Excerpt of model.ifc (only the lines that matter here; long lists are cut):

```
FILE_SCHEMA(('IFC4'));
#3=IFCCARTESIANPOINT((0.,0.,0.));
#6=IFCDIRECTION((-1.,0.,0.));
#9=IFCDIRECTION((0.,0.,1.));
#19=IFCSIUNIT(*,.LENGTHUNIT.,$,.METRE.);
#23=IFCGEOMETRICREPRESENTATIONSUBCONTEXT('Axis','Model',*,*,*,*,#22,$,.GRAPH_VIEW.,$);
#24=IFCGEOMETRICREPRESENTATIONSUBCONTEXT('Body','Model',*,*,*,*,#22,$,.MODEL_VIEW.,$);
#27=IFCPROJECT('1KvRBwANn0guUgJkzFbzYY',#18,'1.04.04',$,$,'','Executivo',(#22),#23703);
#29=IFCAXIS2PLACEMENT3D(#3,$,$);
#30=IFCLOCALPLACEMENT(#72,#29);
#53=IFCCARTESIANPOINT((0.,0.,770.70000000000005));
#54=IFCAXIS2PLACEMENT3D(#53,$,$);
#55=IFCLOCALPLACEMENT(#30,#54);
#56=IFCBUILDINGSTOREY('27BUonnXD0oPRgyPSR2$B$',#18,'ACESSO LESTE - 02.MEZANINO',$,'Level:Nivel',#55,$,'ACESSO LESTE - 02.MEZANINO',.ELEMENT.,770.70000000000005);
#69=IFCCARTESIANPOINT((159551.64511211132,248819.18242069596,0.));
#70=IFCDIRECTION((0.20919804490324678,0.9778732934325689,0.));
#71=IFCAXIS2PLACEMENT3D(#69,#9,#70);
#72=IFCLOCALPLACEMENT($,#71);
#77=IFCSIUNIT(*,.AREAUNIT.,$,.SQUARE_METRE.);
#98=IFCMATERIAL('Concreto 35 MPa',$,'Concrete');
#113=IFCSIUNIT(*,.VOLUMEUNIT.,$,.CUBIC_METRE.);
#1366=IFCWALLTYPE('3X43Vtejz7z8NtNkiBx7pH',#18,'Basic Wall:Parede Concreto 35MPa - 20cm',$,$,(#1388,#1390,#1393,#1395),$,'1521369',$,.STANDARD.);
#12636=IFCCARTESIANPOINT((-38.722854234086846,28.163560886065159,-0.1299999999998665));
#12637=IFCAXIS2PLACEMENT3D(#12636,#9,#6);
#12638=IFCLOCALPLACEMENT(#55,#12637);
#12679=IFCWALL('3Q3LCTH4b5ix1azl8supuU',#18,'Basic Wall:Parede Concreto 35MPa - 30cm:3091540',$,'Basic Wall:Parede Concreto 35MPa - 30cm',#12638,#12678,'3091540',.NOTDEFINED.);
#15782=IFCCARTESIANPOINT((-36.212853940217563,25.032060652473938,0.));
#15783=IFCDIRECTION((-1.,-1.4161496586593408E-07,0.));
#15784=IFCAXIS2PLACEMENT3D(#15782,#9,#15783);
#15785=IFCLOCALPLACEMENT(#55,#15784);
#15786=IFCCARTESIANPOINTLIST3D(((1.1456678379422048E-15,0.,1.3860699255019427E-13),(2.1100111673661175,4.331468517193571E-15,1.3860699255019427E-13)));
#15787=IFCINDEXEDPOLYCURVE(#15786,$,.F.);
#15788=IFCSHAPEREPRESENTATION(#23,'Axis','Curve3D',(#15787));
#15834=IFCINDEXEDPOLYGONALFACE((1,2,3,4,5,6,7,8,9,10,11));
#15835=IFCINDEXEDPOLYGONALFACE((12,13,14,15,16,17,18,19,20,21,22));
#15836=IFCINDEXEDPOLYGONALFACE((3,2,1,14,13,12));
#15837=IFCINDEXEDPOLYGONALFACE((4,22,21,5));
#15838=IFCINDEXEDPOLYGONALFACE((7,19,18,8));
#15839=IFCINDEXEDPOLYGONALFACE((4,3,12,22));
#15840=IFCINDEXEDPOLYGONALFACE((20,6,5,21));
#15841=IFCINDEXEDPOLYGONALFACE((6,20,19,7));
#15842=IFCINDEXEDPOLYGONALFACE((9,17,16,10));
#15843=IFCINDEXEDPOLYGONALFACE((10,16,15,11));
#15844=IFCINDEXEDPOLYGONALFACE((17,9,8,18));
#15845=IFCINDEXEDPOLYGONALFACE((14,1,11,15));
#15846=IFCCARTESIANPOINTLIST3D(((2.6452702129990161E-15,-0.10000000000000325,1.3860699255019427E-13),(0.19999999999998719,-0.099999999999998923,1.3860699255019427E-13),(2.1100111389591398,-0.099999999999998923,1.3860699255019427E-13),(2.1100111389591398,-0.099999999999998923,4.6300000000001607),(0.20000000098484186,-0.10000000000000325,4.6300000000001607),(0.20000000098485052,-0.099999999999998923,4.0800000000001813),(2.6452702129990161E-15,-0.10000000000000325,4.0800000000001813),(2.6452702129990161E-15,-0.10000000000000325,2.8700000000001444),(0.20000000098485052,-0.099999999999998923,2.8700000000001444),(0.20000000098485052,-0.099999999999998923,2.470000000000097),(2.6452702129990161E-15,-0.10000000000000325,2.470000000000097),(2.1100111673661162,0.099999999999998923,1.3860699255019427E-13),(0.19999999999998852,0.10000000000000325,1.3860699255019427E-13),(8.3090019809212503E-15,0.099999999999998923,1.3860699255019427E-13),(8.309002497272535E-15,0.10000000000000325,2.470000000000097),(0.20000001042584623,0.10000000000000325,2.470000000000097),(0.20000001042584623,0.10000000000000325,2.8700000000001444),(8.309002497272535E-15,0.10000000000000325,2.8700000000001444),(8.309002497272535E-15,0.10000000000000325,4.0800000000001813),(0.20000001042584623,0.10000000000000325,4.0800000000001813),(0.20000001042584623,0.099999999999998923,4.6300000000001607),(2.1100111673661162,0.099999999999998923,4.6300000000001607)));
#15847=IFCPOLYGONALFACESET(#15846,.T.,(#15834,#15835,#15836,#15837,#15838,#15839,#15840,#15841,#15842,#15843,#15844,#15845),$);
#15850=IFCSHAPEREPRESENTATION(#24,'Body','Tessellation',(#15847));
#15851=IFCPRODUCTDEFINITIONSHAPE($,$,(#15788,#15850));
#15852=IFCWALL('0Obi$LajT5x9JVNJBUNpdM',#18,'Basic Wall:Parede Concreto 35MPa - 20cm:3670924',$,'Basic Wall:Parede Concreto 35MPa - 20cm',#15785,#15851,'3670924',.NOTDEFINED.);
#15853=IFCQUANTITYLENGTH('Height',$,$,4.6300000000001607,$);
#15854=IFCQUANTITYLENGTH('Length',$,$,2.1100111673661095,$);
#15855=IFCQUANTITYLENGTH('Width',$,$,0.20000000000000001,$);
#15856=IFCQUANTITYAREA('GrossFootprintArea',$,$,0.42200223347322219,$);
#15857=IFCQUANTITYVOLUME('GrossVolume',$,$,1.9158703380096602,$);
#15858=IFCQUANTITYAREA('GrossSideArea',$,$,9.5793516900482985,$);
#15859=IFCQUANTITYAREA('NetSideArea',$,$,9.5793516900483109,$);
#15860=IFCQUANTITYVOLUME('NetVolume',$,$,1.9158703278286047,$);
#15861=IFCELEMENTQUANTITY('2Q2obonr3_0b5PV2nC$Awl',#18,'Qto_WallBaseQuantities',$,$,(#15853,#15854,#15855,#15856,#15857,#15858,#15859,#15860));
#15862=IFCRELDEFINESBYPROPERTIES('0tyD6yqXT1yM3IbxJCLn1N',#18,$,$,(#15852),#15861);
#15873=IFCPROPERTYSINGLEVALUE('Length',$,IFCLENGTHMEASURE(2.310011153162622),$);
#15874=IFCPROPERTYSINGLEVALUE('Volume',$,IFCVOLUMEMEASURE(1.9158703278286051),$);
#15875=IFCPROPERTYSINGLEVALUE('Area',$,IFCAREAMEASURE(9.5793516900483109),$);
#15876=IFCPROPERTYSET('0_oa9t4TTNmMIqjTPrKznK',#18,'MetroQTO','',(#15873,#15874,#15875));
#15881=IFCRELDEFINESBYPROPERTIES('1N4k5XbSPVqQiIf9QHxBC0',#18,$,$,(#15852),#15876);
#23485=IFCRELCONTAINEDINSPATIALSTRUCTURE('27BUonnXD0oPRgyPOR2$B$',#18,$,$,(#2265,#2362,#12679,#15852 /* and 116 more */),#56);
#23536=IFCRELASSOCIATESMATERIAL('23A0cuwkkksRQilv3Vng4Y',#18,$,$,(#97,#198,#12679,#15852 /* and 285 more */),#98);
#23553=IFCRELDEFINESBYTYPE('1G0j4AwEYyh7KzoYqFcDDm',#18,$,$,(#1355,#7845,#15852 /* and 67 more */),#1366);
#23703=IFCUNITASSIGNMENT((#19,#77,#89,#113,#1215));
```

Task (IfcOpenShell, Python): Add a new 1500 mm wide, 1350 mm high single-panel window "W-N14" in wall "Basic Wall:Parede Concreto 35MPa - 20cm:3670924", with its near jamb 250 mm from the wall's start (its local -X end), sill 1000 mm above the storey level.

```python
import numpy as np
import ifcopenshell
import ifcopenshell.api.feature
import ifcopenshell.api.geometry
import ifcopenshell.api.pset
import ifcopenshell.api.root
import ifcopenshell.api.spatial
import ifcopenshell.geom
import ifcopenshell.util.element
import ifcopenshell.util.placement
import ifcopenshell.util.representation
import ifcopenshell.util.shape
import ifcopenshell.util.unit

model = ifcopenshell.open("model.ifc")
unit_scale = ifcopenshell.util.unit.calculate_unit_scale(model)
area_scale = ifcopenshell.util.unit.calculate_unit_scale(model, "AREAUNIT")
volume_scale = ifcopenshell.util.unit.calculate_unit_scale(model, "VOLUMEUNIT")
settings = ifcopenshell.geom.settings()


def volume(element):
    """Net volume in cubic metres, openings subtracted."""
    shape = ifcopenshell.geom.create_shape(settings, element)
    return ifcopenshell.util.shape.get_volume(shape.geometry)


wall = model.by_id(15852)
storey = ifcopenshell.util.element.get_container(wall, ifc_class="IfcBuildingStorey")
context = ifcopenshell.util.representation.get_context(model, "Model", "Body", "MODEL_VIEW")
before = volume(wall)

width, height, from_end, sill = 1.5, 1.35, 0.25, 1  # metres

# The wall runs along its own X axis, and the end named is its -X end.
wall_shape = ifcopenshell.geom.create_shape(settings, wall)
x, y, z = ifcopenshell.util.shape.get_vertices(wall_shape.geometry).T
start = x.min() + from_end
face, thickness = float(y.min()), float(y.max() - y.min())
wall_matrix = ifcopenshell.util.placement.get_local_placement(wall.ObjectPlacement)
level = ifcopenshell.util.placement.get_local_placement(storey.ObjectPlacement)[2, 3]


def in_wall(x, y):
    """Placement at x, y metres in the wall's axes, at sill height."""
    matrix = wall_matrix.copy()
    matrix[:, 3] = wall_matrix @ np.array([x / unit_scale, y / unit_scale, 0.0, 1.0])
    matrix[2, 3] = level + sill / unit_scale
    return matrix


# Opening: a box that overshoots both wall faces by 50 mm.
opening = ifcopenshell.api.root.create_entity(model, ifc_class="IfcOpeningElement", predefined_type="OPENING")
box = ifcopenshell.api.geometry.add_wall_representation(
    model, context=context, length=width, height=height, thickness=thickness + 0.1
)
ifcopenshell.api.geometry.assign_representation(model, product=opening, representation=box)
ifcopenshell.api.geometry.edit_object_placement(model, product=opening, matrix=in_wall(start, face - 0.05), is_si=False)
ifcopenshell.api.feature.add_feature(model, feature=opening, element=wall)

window = ifcopenshell.api.root.create_entity(model, ifc_class="IfcWindow", name="W-N14", predefined_type="WINDOW")
window.OverallWidth, window.OverallHeight = width / unit_scale, height / unit_scale
window.PartitioningType = "SINGLE_PANEL"
body = ifcopenshell.api.geometry.add_window_representation(
    model,
    context=context,
    overall_width=window.OverallWidth,
    overall_height=window.OverallHeight,
    partition_type="SINGLE_PANEL",
)
ifcopenshell.api.geometry.assign_representation(model, product=window, representation=body)
ifcopenshell.api.spatial.assign_container(model, products=[window], relating_structure=storey)
ifcopenshell.api.feature.add_filling(model, opening=opening, element=window)

# Centre the window in the wall's thickness.
ifcopenshell.api.geometry.edit_object_placement(model, product=window, matrix=in_wall(start, face), is_si=False)
window_shape = ifcopenshell.geom.create_shape(settings, window)
depth = ifcopenshell.util.shape.get_vertices(window_shape.geometry)[:, 1]
offset = face + thickness / 2 - (depth.min() + depth.max()) / 2
ifcopenshell.api.geometry.edit_object_placement(model, product=window, matrix=in_wall(start, offset), is_si=False)

after = volume(wall)

# Update the wall's stored quantities.
qto = model.by_id(ifcopenshell.util.element.get_pset(wall, "Qto_WallBaseQuantities", should_inherit=False)["id"])
ifcopenshell.api.pset.edit_qto(model, qto=qto, properties={
    "NetSideArea": after / thickness / area_scale,
    "NetVolume": after / volume_scale,
})
pset = model.by_id(ifcopenshell.util.element.get_pset(wall, "MetroQTO", should_inherit=False)["id"])
ifcopenshell.api.pset.edit_pset(model, pset=pset, properties={
    "Volume": model.create_entity("IfcVolumeMeasure", after / volume_scale),
    "Area": model.create_entity("IfcAreaMeasure", after / thickness / area_scale),
})

print(f"wall volume {before:.3f} -> {after:.3f} m3")

model.write("model_v2.ifc")
```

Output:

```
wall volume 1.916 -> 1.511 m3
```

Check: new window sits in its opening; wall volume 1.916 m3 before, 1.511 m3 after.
